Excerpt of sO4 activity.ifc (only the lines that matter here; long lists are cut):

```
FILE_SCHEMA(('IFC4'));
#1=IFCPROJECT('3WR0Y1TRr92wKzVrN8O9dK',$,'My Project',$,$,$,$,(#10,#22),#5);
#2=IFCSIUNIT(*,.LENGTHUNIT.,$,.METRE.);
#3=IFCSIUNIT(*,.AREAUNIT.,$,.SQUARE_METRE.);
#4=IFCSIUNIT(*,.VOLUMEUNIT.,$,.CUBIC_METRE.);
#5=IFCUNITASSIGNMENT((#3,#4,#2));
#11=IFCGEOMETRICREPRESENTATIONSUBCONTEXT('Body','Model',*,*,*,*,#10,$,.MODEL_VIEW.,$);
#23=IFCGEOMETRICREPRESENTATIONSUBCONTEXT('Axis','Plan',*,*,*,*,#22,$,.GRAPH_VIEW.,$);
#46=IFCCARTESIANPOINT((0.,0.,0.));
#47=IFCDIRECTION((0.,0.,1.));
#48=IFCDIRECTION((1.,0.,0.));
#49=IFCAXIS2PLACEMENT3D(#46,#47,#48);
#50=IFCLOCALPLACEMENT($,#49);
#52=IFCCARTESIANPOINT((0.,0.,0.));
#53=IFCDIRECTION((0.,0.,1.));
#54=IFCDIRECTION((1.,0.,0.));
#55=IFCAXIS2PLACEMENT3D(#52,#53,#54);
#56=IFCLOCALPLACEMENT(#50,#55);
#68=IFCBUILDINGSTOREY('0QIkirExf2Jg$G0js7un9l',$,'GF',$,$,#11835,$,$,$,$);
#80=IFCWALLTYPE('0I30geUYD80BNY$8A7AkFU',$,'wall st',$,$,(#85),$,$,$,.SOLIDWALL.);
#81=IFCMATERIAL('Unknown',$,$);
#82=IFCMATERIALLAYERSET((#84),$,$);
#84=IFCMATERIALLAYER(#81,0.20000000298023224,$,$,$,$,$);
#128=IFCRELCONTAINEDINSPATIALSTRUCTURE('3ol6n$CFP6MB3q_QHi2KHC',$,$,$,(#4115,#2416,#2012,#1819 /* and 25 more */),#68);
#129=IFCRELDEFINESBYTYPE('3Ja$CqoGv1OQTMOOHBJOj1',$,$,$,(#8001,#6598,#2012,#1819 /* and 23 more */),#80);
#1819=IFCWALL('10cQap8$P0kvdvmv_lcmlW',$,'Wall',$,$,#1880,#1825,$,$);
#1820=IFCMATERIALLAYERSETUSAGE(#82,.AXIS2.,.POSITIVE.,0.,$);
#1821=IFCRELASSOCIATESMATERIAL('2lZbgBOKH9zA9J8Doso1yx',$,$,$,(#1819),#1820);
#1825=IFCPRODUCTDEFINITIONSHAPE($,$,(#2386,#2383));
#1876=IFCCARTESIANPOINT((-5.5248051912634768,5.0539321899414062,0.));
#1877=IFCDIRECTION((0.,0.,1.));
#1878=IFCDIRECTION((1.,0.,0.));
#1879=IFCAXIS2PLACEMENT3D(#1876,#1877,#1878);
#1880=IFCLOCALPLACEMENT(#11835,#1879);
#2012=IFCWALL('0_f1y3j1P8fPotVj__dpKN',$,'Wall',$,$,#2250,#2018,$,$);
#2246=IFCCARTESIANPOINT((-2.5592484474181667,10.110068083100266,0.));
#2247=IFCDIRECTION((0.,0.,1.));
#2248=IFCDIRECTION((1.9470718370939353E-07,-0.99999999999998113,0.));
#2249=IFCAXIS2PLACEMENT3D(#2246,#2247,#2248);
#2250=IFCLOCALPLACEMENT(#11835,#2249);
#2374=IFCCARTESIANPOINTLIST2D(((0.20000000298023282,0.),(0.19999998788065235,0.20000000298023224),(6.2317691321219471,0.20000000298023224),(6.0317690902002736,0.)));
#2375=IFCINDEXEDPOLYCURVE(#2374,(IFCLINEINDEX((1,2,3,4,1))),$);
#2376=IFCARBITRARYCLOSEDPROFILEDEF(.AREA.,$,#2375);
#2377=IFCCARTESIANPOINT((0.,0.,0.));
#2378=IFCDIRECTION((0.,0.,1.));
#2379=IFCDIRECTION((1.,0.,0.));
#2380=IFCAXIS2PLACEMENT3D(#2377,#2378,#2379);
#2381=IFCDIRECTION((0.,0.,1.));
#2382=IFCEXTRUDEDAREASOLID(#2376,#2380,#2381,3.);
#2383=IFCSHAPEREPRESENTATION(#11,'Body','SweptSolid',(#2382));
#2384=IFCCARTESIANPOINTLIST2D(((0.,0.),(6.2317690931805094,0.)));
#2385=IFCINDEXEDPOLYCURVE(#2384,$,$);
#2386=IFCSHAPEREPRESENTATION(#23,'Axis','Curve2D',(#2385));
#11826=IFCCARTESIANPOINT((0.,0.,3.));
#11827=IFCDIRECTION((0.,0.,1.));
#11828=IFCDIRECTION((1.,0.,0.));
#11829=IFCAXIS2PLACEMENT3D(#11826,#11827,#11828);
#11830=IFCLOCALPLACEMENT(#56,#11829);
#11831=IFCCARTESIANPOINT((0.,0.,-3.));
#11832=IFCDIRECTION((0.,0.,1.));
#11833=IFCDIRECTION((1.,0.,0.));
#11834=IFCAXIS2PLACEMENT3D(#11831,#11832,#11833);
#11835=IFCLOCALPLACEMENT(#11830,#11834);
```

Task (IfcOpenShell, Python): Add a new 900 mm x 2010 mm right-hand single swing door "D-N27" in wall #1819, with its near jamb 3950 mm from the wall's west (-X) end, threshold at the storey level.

```python
import numpy as np
import ifcopenshell
import ifcopenshell.api.feature
import ifcopenshell.api.geometry
import ifcopenshell.api.root
import ifcopenshell.api.spatial
import ifcopenshell.geom
import ifcopenshell.util.element
import ifcopenshell.util.placement
import ifcopenshell.util.representation
import ifcopenshell.util.shape
import ifcopenshell.util.unit

model = ifcopenshell.open("sO4 activity.ifc")
unit_scale = ifcopenshell.util.unit.calculate_unit_scale(model)
settings = ifcopenshell.geom.settings()


def volume(element):
    """Net volume in cubic metres, openings subtracted."""
    shape = ifcopenshell.geom.create_shape(settings, element)
    return ifcopenshell.util.shape.get_volume(shape.geometry)


wall = model.by_guid("10cQap8$P0kvdvmv_lcmlW")
storey = ifcopenshell.util.element.get_container(wall, ifc_class="IfcBuildingStorey")
context = ifcopenshell.util.representation.get_context(model, "Model", "Body", "MODEL_VIEW")
before = volume(wall)

width, height, from_end, sill = 0.9, 2.01, 3.95, 0.0  # metres

# The wall runs along its own X axis, and the end named is its -X end.
wall_shape = ifcopenshell.geom.create_shape(settings, wall)
x, y, z = ifcopenshell.util.shape.get_vertices(wall_shape.geometry).T
start = x.min() + from_end
face, thickness = float(y.min()), float(y.max() - y.min())
wall_matrix = ifcopenshell.util.placement.get_local_placement(wall.ObjectPlacement)
level = ifcopenshell.util.placement.get_local_placement(storey.ObjectPlacement)[2, 3]


def in_wall(x, y):
    """Placement at x, y metres in the wall's axes, at sill height."""
    matrix = wall_matrix.copy()
    matrix[:, 3] = wall_matrix @ np.array([x / unit_scale, y / unit_scale, 0.0, 1.0])
    matrix[2, 3] = level + sill / unit_scale
    return matrix


# Opening: a box that overshoots both wall faces by 50 mm.
opening = ifcopenshell.api.root.create_entity(model, ifc_class="IfcOpeningElement", predefined_type="OPENING")
box = ifcopenshell.api.geometry.add_wall_representation(
    model, context=context, length=width, height=height, thickness=thickness + 0.1
)
ifcopenshell.api.geometry.assign_representation(model, product=opening, representation=box)
ifcopenshell.api.geometry.edit_object_placement(model, product=opening, matrix=in_wall(start, face - 0.05), is_si=False)
ifcopenshell.api.feature.add_feature(model, feature=opening, element=wall)

door = ifcopenshell.api.root.create_entity(model, ifc_class="IfcDoor", name="D-N27", predefined_type="DOOR")
door.OverallWidth, door.OverallHeight = width / unit_scale, height / unit_scale
door.OperationType = "SINGLE_SWING_RIGHT"
body = ifcopenshell.api.geometry.add_door_representation(
    model,
    context=context,
    overall_width=door.OverallWidth,
    overall_height=door.OverallHeight,
    operation_type="SINGLE_SWING_RIGHT",
    lining_properties={"LiningDepth": thickness / unit_scale, "ThresholdDepth": thickness / unit_scale},
)
ifcopenshell.api.geometry.assign_representation(model, product=door, representation=body)
ifcopenshell.api.spatial.assign_container(model, products=[door], relating_structure=storey)
ifcopenshell.api.feature.add_filling(model, opening=opening, element=door)

# The lining spans the wall, so the door starts at the wall face.
ifcopenshell.api.geometry.edit_object_placement(model, product=door, matrix=in_wall(start, face), is_si=False)

after = volume(wall)

print(f"wall volume {before:.3f} -> {after:.3f} m3")

model.write("sO4 activity-out.ifc")
```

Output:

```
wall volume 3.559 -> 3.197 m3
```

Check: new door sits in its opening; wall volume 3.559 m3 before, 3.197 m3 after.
